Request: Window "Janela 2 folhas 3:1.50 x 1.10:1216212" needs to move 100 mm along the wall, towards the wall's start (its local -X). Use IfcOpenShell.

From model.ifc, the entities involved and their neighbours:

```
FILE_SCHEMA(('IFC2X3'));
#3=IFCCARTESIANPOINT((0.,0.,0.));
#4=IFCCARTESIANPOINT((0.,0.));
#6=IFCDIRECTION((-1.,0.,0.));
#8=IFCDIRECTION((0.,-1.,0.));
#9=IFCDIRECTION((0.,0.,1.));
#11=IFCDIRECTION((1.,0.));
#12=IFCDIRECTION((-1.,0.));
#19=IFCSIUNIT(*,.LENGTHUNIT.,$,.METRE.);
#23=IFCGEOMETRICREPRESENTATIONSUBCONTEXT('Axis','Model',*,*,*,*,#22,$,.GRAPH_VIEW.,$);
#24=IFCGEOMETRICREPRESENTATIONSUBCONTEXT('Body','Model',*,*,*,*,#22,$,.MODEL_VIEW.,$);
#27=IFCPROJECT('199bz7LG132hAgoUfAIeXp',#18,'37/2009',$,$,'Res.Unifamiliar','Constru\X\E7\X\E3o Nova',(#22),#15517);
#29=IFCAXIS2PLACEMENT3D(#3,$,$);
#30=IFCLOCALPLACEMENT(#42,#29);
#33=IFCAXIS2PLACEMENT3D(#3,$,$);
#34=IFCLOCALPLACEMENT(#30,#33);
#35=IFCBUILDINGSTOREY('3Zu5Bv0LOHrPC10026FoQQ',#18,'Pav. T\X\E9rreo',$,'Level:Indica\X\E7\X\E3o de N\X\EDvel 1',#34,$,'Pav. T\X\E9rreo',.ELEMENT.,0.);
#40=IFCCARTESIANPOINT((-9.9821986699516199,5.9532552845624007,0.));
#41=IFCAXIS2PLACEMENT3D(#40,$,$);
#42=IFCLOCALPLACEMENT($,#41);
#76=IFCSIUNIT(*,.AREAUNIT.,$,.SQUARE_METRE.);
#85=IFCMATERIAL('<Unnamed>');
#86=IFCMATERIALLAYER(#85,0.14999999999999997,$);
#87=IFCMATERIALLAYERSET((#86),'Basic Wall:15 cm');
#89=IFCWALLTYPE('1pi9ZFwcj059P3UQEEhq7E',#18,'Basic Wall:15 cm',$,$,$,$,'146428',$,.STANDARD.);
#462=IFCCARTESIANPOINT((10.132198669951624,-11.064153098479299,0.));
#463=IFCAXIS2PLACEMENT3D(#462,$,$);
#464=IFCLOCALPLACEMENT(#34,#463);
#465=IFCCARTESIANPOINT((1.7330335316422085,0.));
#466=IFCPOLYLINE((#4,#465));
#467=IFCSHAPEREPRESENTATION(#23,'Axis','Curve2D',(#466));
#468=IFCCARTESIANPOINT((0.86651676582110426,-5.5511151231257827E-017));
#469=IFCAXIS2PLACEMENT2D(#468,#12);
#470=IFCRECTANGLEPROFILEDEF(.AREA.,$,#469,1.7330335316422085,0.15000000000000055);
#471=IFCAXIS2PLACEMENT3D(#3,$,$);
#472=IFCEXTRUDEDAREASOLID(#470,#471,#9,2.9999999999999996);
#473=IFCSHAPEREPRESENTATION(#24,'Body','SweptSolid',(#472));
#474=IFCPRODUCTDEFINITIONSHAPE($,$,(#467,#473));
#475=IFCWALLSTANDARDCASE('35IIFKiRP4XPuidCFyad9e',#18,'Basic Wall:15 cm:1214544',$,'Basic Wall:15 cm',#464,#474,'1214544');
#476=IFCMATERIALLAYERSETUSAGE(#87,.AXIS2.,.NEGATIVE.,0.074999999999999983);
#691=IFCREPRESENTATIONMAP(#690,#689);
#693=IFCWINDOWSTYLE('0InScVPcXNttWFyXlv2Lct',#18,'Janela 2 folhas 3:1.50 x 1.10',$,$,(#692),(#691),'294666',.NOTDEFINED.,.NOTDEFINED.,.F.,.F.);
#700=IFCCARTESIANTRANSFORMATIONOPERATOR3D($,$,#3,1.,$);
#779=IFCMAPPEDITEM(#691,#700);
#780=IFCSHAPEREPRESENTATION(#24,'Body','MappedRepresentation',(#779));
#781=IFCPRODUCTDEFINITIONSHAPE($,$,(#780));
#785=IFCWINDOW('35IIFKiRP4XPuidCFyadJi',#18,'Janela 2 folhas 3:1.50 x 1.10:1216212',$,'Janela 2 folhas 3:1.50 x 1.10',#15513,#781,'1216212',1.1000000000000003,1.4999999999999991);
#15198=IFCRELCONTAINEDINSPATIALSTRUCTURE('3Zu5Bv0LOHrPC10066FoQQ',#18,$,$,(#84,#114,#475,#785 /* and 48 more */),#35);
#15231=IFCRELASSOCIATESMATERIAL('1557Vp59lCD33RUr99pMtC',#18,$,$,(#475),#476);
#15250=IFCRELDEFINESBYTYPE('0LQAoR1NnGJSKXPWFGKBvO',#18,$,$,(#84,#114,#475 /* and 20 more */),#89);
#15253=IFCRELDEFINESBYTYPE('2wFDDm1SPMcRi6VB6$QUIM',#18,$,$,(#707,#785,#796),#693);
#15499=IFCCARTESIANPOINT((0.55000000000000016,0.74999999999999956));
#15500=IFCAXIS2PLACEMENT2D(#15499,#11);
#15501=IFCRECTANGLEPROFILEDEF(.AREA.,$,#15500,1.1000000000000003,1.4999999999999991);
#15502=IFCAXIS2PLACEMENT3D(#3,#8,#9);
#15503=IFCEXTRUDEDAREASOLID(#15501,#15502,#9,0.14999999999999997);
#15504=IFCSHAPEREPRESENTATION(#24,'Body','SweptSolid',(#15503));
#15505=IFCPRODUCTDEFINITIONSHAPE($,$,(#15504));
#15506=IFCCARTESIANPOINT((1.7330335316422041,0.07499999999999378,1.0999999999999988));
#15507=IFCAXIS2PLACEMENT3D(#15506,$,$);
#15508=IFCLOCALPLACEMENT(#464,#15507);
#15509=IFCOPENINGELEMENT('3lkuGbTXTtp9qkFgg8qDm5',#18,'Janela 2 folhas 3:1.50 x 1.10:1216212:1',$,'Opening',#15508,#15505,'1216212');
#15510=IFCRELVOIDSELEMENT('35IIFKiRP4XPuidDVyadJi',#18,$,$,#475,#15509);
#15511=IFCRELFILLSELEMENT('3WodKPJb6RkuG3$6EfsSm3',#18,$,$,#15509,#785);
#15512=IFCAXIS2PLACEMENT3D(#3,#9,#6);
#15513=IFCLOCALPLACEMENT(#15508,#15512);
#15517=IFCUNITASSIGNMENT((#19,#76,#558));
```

```python
import ifcopenshell
import ifcopenshell.api.geometry
import ifcopenshell.util.placement

model = ifcopenshell.open("model.ifc")

window = model.by_guid("35IIFKiRP4XPuidCFyadJi")
opening = window.FillsVoids[0].RelatingOpeningElement
wall = opening.VoidsElements[0].RelatingBuildingElement

wall_matrix = ifcopenshell.util.placement.get_local_placement(wall.ObjectPlacement)
shift = wall_matrix[:3, 0] * -0.1
before = ifcopenshell.util.placement.get_local_placement(window.ObjectPlacement)[:3, 3].copy()

# The window is placed relative to its opening, so it follows when the opening moves.
matrix = ifcopenshell.util.placement.get_local_placement(opening.ObjectPlacement)
matrix[:3, 3] += shift
ifcopenshell.api.geometry.edit_object_placement(
    model, product=opening, matrix=matrix, is_si=False, should_transform_children=True
)

after = ifcopenshell.util.placement.get_local_placement(window.ObjectPlacement)[:3, 3]
print("window moved by", (after - before).round(3) + 0.0)

model.write("model-out.ifc")
```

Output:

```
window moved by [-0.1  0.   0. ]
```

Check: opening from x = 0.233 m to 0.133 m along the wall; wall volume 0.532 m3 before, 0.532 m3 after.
